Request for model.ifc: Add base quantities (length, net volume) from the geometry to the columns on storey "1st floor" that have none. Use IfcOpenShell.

First a look at what the model holds.

```python
import ifcopenshell
import ifcopenshell.util.element
import ifcopenshell.util.unit

model = ifcopenshell.open("model.ifc")
print(model.schema)
for unit_type in ("LENGTHUNIT", "AREAUNIT", "VOLUMEUNIT"):
    print(unit_type, ifcopenshell.util.unit.calculate_unit_scale(model, unit_type))
storey = next(s for s in model.by_type("IfcBuildingStorey") if s.Name == "1st floor")
columns = [e for e in ifcopenshell.util.element.get_decomposition(storey) if e.is_a("IfcColumn")]
for e in sorted(columns, key=lambda e: e.id()):
    print(e.id(), e.is_a(), e.Name, list(ifcopenshell.util.element.get_psets(e, qtos_only=True)), sep=" | ")
```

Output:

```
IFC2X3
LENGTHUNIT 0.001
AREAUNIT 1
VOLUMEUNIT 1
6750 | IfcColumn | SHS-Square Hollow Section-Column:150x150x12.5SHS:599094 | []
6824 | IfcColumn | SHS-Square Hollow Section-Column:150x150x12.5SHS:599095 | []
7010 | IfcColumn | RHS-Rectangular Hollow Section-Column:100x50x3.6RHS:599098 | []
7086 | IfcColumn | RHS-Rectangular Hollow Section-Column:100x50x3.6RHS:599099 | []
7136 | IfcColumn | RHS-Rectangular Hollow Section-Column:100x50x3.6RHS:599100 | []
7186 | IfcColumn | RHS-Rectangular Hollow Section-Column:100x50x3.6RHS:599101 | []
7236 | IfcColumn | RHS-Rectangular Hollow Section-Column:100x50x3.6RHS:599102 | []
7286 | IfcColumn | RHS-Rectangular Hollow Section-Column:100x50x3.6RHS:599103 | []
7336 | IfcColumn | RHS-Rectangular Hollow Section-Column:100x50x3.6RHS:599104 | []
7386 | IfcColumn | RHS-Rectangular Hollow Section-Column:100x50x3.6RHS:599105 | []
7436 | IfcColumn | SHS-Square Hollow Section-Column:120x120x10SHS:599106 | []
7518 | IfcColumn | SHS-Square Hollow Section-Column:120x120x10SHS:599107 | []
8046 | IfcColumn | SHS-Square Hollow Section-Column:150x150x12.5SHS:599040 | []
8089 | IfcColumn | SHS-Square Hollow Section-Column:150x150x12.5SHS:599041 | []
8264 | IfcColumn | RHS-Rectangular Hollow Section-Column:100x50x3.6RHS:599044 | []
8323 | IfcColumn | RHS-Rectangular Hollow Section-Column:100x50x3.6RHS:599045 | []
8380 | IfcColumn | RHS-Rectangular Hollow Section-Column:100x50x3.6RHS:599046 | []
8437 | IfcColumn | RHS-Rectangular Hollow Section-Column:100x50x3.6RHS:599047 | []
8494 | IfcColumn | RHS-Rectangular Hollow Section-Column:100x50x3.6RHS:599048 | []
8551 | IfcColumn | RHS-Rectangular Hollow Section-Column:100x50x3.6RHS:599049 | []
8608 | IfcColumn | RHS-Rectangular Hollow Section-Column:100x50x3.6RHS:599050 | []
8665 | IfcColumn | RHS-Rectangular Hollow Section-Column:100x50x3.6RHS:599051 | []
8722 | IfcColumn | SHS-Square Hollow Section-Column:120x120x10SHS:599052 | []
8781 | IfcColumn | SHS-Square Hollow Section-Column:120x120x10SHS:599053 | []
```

```python
import ifcopenshell
import ifcopenshell.api.pset
import ifcopenshell.geom
import ifcopenshell.util.element
import ifcopenshell.util.shape
import ifcopenshell.util.unit

model = ifcopenshell.open("model.ifc")
unit_scale = ifcopenshell.util.unit.calculate_unit_scale(model)
volume_scale = ifcopenshell.util.unit.calculate_unit_scale(model, "VOLUMEUNIT")
settings = ifcopenshell.geom.settings()

storey = next(s for s in model.by_type("IfcBuildingStorey") if s.Name == "1st floor")
columns = [e for e in ifcopenshell.util.element.get_decomposition(storey) if e.is_a("IfcColumn")]

for e in sorted(columns, key=lambda e: e.id()):
    if ifcopenshell.util.element.get_psets(e, qtos_only=True, should_inherit=False):
        continue
    # Geometry comes back in metres, in the element's own axes.
    shape = ifcopenshell.geom.create_shape(settings, e)
    values = {
        "Length": ifcopenshell.util.shape.get_z(shape.geometry) / unit_scale,
        "NetVolume": ifcopenshell.util.shape.get_volume(shape.geometry) / volume_scale,
    }
    qto = ifcopenshell.api.pset.add_qto(model, product=e, name="BaseQuantities")
    ifcopenshell.api.pset.edit_qto(model, qto=qto, properties=values)
    print(e.id(), {k: round(v, 3) for k, v in values.items()})

model.write("model_v2.ifc")
```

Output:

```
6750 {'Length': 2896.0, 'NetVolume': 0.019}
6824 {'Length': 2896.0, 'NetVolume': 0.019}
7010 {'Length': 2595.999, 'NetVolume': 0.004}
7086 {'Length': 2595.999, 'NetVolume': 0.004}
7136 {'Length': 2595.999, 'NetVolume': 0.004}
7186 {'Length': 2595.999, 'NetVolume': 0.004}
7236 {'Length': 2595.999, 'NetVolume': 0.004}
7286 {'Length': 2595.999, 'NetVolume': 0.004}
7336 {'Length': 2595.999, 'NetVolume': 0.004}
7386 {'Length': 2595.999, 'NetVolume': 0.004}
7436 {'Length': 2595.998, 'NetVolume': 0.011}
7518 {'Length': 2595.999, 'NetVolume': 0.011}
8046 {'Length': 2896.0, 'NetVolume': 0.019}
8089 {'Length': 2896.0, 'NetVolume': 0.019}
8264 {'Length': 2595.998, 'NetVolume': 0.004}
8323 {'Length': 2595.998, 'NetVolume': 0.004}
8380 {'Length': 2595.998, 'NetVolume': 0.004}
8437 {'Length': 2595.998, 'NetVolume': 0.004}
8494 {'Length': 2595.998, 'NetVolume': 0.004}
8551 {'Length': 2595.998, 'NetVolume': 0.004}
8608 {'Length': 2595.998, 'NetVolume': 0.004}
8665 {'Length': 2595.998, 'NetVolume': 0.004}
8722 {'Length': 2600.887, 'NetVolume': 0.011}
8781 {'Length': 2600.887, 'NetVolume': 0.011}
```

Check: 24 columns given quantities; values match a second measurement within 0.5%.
